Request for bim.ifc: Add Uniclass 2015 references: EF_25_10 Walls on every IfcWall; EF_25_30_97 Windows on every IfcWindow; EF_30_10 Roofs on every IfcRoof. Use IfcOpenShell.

First a look at what the model holds.

```python
import ifcopenshell

model = ifcopenshell.open("bim.ifc")
print(model.schema)
print("classifications:", [c.Name for c in model.by_type("IfcClassification")])
for ifc_class in ("IfcDoor", "IfcRoof", "IfcStair", "IfcWall", "IfcWindow"):
    print(ifc_class, len(model.by_type(ifc_class)))
```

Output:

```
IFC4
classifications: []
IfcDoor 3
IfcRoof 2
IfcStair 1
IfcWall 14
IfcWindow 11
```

```python
import ifcopenshell
import ifcopenshell.api.classification

model = ifcopenshell.open("bim.ifc")

system = ifcopenshell.api.classification.add_classification(model, classification="Uniclass 2015")

codes = {
    "IfcWall": ("EF_25_10", "Walls"),
    "IfcWindow": ("EF_25_30_97", "Windows"),
    "IfcRoof": ("EF_30_10", "Roofs"),
}
for ifc_class, (code, name) in codes.items():
    products = model.by_type(ifc_class)
    ifcopenshell.api.classification.add_reference(
        model, products=products, classification=system, identification=code, name=name
    )
    print(code, len(products))

model.write("bim_v2.ifc")
```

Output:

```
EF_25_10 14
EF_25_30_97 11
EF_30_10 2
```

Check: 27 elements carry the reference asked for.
